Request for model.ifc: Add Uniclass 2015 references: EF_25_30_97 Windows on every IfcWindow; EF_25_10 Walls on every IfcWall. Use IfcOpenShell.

First a look at what the model holds.

```python
import ifcopenshell

model = ifcopenshell.open("model.ifc")
print(model.schema)
print("classifications:", [c.Name for c in model.by_type("IfcClassification")])
for ifc_class in ("IfcDoor", "IfcRoof", "IfcStair", "IfcWall", "IfcWindow"):
    print(ifc_class, len(model.by_type(ifc_class)))
```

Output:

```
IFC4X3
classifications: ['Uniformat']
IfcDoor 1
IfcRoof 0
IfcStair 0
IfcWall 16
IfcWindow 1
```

```python
import ifcopenshell
import ifcopenshell.api.classification

model = ifcopenshell.open("model.ifc")

system = ifcopenshell.api.classification.add_classification(model, classification="Uniclass 2015")

codes = {
    "IfcWindow": ("EF_25_30_97", "Windows"),
    "IfcWall": ("EF_25_10", "Walls"),
}
for ifc_class, (code, name) in codes.items():
    products = model.by_type(ifc_class)
    ifcopenshell.api.classification.add_reference(
        model, products=products, classification=system, identification=code, name=name
    )
    print(code, len(products))

model.write("model_rev.ifc")
```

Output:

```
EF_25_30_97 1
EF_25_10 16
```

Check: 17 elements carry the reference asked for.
